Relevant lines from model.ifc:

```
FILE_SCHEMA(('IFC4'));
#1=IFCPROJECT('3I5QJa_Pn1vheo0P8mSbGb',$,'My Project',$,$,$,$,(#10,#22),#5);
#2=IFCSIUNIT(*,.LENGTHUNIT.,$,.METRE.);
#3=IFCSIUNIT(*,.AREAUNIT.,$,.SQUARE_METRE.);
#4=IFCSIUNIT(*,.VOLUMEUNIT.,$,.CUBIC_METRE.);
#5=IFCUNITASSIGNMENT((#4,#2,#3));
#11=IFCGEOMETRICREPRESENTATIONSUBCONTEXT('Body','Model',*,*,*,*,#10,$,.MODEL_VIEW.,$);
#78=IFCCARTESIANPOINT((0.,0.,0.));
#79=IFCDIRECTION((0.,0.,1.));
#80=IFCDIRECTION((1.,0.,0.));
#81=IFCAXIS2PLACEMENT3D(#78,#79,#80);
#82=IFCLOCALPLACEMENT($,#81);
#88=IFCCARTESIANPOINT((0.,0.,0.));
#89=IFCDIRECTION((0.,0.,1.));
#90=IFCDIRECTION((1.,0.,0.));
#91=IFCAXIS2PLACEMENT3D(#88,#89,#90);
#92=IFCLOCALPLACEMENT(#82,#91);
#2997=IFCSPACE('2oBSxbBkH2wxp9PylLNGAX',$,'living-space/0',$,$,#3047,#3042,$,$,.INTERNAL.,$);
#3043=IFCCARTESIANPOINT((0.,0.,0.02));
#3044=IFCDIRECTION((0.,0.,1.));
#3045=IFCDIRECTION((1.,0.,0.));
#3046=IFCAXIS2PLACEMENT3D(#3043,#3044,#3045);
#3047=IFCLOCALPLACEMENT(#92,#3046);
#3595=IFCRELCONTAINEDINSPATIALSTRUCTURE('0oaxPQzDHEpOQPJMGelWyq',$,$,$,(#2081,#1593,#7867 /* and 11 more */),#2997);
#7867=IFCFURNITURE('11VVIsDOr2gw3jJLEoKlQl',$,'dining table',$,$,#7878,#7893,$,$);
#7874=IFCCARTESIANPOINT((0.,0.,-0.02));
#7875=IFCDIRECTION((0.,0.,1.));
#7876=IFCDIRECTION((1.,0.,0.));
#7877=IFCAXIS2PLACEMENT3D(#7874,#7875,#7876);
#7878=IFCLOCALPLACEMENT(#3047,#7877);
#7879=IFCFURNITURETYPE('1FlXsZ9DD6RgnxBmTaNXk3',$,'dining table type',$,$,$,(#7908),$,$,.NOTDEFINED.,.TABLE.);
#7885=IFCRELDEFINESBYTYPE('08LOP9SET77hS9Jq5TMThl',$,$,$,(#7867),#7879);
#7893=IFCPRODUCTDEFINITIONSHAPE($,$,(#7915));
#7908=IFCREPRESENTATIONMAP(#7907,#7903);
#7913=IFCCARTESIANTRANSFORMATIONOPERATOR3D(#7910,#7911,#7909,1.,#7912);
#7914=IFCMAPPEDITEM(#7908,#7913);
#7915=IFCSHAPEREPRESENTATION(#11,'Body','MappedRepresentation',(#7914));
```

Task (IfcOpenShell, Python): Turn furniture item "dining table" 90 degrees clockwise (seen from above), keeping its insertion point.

```python
import ifcopenshell
import ifcopenshell.api.geometry
import ifcopenshell.util.placement

model = ifcopenshell.open("model.ifc")

item = model.by_id(7867)
matrix = ifcopenshell.util.placement.get_local_placement(item.ObjectPlacement)
matrix = matrix @ ifcopenshell.util.placement.rotation(-90, "Z")
ifcopenshell.api.geometry.edit_object_placement(model, product=item, matrix=matrix, is_si=False)

print(ifcopenshell.util.placement.get_local_placement(item.ObjectPlacement).round(3) + 0.0)

model.write("model-out.ifc")
```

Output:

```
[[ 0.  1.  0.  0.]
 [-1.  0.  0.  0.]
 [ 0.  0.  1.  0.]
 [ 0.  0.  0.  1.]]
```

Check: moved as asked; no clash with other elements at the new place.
